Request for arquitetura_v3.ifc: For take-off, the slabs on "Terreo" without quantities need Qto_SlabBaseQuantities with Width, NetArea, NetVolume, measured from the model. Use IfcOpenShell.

First a look at what the model holds.

```python
import ifcopenshell
import ifcopenshell.util.element
import ifcopenshell.util.unit

model = ifcopenshell.open("arquitetura_v3.ifc")
print(model.schema)
for unit_type in ("LENGTHUNIT", "AREAUNIT", "VOLUMEUNIT"):
    print(unit_type, ifcopenshell.util.unit.calculate_unit_scale(model, unit_type))
storey = next(s for s in model.by_type("IfcBuildingStorey") if s.Name == "Terreo")
slabs = [e for e in ifcopenshell.util.element.get_decomposition(storey) if e.is_a("IfcSlab")]
for e in sorted(slabs, key=lambda e: e.id()):
    print(e.id(), e.is_a(), e.Name, list(ifcopenshell.util.element.get_psets(e, qtos_only=True)), sep=" | ")
```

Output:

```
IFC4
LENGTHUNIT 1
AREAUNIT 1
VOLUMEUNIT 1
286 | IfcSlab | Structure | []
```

```python
import ifcopenshell
import ifcopenshell.api.pset
import ifcopenshell.geom
import ifcopenshell.util.element
import ifcopenshell.util.shape
import ifcopenshell.util.unit

model = ifcopenshell.open("arquitetura_v3.ifc")
unit_scale = ifcopenshell.util.unit.calculate_unit_scale(model)
area_scale = ifcopenshell.util.unit.calculate_unit_scale(model, "AREAUNIT")
volume_scale = ifcopenshell.util.unit.calculate_unit_scale(model, "VOLUMEUNIT")
settings = ifcopenshell.geom.settings()

storey = next(s for s in model.by_type("IfcBuildingStorey") if s.Name == "Terreo")
slabs = [e for e in ifcopenshell.util.element.get_decomposition(storey) if e.is_a("IfcSlab")]

for e in sorted(slabs, key=lambda e: e.id()):
    if ifcopenshell.util.element.get_psets(e, qtos_only=True, should_inherit=False):
        continue
    # Geometry comes back in metres, in the element's own axes.
    shape = ifcopenshell.geom.create_shape(settings, e)
    values = {
        "Width": ifcopenshell.util.shape.get_z(shape.geometry) / unit_scale,
        "NetArea": ifcopenshell.util.shape.get_footprint_area(shape.geometry) / area_scale,
        "NetVolume": ifcopenshell.util.shape.get_volume(shape.geometry) / volume_scale,
    }
    qto = ifcopenshell.api.pset.add_qto(model, product=e, name="Qto_SlabBaseQuantities")
    ifcopenshell.api.pset.edit_qto(model, qto=qto, properties=values)
    print(e.id(), {k: round(v, 3) for k, v in values.items()})

model.write("arquitetura_v3_v2.ifc")
```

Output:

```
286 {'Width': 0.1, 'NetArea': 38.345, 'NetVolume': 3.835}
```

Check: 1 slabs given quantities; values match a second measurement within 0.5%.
